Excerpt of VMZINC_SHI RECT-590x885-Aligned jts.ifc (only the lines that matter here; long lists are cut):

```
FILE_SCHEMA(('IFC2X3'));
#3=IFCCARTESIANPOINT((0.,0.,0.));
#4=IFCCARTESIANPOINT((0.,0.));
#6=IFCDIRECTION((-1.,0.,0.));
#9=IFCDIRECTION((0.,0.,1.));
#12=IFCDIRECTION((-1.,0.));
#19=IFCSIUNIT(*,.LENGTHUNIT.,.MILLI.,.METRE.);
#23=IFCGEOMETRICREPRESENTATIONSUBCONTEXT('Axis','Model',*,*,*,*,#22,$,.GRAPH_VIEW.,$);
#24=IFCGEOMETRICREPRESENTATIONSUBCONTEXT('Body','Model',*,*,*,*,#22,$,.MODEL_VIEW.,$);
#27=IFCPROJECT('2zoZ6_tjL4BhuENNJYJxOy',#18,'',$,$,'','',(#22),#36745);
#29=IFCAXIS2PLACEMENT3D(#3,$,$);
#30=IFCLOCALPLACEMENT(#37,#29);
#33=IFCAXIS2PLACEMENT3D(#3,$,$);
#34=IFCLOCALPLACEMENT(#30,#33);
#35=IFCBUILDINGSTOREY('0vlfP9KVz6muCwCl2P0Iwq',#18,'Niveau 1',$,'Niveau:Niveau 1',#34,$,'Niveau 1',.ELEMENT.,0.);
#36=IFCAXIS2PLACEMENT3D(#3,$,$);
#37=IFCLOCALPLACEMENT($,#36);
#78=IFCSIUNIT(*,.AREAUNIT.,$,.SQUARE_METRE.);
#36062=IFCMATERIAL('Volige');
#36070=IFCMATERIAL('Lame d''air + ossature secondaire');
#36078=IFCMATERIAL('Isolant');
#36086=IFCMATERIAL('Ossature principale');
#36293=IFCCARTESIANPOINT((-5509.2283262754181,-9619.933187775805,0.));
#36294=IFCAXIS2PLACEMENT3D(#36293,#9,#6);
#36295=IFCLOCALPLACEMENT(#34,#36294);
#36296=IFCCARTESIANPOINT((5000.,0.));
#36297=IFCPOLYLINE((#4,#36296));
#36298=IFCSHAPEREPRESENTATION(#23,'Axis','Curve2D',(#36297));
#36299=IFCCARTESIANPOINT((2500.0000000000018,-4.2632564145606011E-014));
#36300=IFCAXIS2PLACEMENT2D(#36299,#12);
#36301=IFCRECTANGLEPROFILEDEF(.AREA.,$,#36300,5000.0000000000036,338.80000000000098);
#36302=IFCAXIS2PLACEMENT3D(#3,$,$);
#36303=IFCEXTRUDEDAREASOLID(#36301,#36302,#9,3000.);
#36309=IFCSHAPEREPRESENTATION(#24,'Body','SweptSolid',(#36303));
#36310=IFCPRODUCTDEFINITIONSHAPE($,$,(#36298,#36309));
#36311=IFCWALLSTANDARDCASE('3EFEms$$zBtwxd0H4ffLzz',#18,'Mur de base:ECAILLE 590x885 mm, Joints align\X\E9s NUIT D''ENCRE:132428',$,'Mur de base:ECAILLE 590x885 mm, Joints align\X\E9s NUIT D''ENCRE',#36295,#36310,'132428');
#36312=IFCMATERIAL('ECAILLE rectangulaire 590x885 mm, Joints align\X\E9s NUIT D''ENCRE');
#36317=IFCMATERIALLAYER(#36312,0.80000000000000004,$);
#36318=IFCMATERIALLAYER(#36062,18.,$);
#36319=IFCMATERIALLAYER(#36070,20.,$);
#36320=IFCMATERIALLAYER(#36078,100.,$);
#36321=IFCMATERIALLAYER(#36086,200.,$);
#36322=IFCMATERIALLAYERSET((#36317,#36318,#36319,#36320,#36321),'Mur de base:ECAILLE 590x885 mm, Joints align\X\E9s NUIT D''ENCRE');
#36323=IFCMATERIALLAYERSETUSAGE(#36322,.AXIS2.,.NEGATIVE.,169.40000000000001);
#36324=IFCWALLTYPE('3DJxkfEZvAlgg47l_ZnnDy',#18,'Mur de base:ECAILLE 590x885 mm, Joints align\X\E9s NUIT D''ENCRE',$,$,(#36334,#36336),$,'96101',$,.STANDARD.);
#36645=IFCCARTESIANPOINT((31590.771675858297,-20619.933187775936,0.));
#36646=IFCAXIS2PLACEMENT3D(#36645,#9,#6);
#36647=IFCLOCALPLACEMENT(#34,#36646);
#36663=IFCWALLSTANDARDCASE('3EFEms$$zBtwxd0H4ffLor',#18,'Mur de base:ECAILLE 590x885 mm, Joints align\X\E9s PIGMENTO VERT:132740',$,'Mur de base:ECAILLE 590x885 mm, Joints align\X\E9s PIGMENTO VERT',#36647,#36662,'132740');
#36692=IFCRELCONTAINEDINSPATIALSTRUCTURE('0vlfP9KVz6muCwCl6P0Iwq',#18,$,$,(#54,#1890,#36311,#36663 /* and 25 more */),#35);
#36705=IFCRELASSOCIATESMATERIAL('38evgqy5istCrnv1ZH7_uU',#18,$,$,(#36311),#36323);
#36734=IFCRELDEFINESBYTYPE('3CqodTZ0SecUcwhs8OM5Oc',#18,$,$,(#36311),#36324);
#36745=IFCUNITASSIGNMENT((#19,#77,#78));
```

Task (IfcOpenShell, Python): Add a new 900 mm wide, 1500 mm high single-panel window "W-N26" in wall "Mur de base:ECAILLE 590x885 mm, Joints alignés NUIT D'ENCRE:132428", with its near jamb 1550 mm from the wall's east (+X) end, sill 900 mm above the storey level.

```python
import numpy as np
import ifcopenshell
import ifcopenshell.api.feature
import ifcopenshell.api.geometry
import ifcopenshell.api.root
import ifcopenshell.api.spatial
import ifcopenshell.api.type
import ifcopenshell.geom
import ifcopenshell.util.element
import ifcopenshell.util.placement
import ifcopenshell.util.representation
import ifcopenshell.util.shape
import ifcopenshell.util.unit

model = ifcopenshell.open("VMZINC_SHI RECT-590x885-Aligned jts.ifc")
unit_scale = ifcopenshell.util.unit.calculate_unit_scale(model)
settings = ifcopenshell.geom.settings()


def volume(element):
    """Net volume in cubic metres, openings subtracted."""
    shape = ifcopenshell.geom.create_shape(settings, element)
    return ifcopenshell.util.shape.get_volume(shape.geometry)


wall = model.by_id(36311)
storey = ifcopenshell.util.element.get_container(wall, ifc_class="IfcBuildingStorey")
context = ifcopenshell.util.representation.get_context(model, "Model", "Body", "MODEL_VIEW")
before = volume(wall)

width, height, from_end, sill = 0.9, 1.5, 1.55, 0.9  # metres

# The wall runs along its own X axis, and the end named is its -X end.
wall_shape = ifcopenshell.geom.create_shape(settings, wall)
x, y, z = ifcopenshell.util.shape.get_vertices(wall_shape.geometry).T
start = x.min() + from_end
face, thickness = float(y.min()), float(y.max() - y.min())
wall_matrix = ifcopenshell.util.placement.get_local_placement(wall.ObjectPlacement)
level = ifcopenshell.util.placement.get_local_placement(storey.ObjectPlacement)[2, 3]


def in_wall(x, y):
    """Placement at x, y metres in the wall's axes, at sill height."""
    matrix = wall_matrix.copy()
    matrix[:, 3] = wall_matrix @ np.array([x / unit_scale, y / unit_scale, 0.0, 1.0])
    matrix[2, 3] = level + sill / unit_scale
    return matrix


# Opening: a box that overshoots both wall faces by 50 mm.
opening = ifcopenshell.api.root.create_entity(model, ifc_class="IfcOpeningElement")
box = ifcopenshell.api.geometry.add_wall_representation(
    model, context=context, length=width, height=height, thickness=thickness + 0.1
)
ifcopenshell.api.geometry.assign_representation(model, product=opening, representation=box)
ifcopenshell.api.geometry.edit_object_placement(model, product=opening, matrix=in_wall(start, face - 0.05), is_si=False)
ifcopenshell.api.feature.add_feature(model, feature=opening, element=wall)

window = ifcopenshell.api.root.create_entity(model, ifc_class="IfcWindow", name="W-N26")
window.OverallWidth, window.OverallHeight = width / unit_scale, height / unit_scale
body = ifcopenshell.api.geometry.add_window_representation(
    model,
    context=context,
    overall_width=window.OverallWidth,
    overall_height=window.OverallHeight,
    partition_type="SINGLE_PANEL",
)
ifcopenshell.api.geometry.assign_representation(model, product=window, representation=body)
ifcopenshell.api.spatial.assign_container(model, products=[window], relating_structure=storey)
fills = ifcopenshell.api.feature.add_filling(model, opening=opening, element=window)
fills.OwnerHistory = window.OwnerHistory  # required in IFC2X3

# IFC2X3 keeps the operation on the window style.
style = ifcopenshell.api.root.create_entity(model, ifc_class="IfcWindowStyle", name="W-N26")
style.OperationType, style.ConstructionType = "SINGLE_PANEL", "NOTDEFINED"
style.ParameterTakesPrecedence = style.Sizeable = False
ifcopenshell.api.type.assign_type(model, related_objects=[window], relating_type=style)

# Centre the window in the wall's thickness.
ifcopenshell.api.geometry.edit_object_placement(model, product=window, matrix=in_wall(start, face), is_si=False)
window_shape = ifcopenshell.geom.create_shape(settings, window)
depth = ifcopenshell.util.shape.get_vertices(window_shape.geometry)[:, 1]
offset = face + thickness / 2 - (depth.min() + depth.max()) / 2
ifcopenshell.api.geometry.edit_object_placement(model, product=window, matrix=in_wall(start, offset), is_si=False)

after = volume(wall)

print(f"wall volume {before:.3f} -> {after:.3f} m3")

model.write("VMZINC_SHI RECT-590x885-Aligned jts-out.ifc")
```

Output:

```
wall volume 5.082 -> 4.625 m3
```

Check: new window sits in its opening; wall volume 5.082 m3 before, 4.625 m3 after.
